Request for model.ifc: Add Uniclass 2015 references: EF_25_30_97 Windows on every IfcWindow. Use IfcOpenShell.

First a look at what the model holds.

```python
import ifcopenshell

model = ifcopenshell.open("model.ifc")
print(model.schema)
print("classifications:", [c.Name for c in model.by_type("IfcClassification")])
for ifc_class in ("IfcDoor", "IfcRoof", "IfcStair", "IfcWall", "IfcWindow"):
    print(ifc_class, len(model.by_type(ifc_class)))
```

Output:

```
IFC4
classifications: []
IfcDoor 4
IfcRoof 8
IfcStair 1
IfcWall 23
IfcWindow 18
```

```python
import ifcopenshell
import ifcopenshell.api.classification

model = ifcopenshell.open("model.ifc")

system = ifcopenshell.api.classification.add_classification(model, classification="Uniclass 2015")

codes = {
    "IfcWindow": ("EF_25_30_97", "Windows"),
}
for ifc_class, (code, name) in codes.items():
    products = model.by_type(ifc_class)
    ifcopenshell.api.classification.add_reference(
        model, products=products, classification=system, identification=code, name=name
    )
    print(code, len(products))

model.write("model-out.ifc")
```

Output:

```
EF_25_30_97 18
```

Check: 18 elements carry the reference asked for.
